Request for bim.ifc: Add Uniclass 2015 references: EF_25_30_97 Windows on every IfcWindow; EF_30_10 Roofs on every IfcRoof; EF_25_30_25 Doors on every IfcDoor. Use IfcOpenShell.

First a look at what the model holds.

```python
import ifcopenshell

model = ifcopenshell.open("bim.ifc")
print(model.schema)
print("classifications:", [c.Name for c in model.by_type("IfcClassification")])
for ifc_class in ("IfcDoor", "IfcRoof", "IfcStair", "IfcWall", "IfcWindow"):
    print(ifc_class, len(model.by_type(ifc_class)))
```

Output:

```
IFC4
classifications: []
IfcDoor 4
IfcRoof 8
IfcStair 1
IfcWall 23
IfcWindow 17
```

```python
import ifcopenshell
import ifcopenshell.api.classification

model = ifcopenshell.open("bim.ifc")

system = ifcopenshell.api.classification.add_classification(model, classification="Uniclass 2015")

codes = {
    "IfcWindow": ("EF_25_30_97", "Windows"),
    "IfcRoof": ("EF_30_10", "Roofs"),
    "IfcDoor": ("EF_25_30_25", "Doors"),
}
for ifc_class, (code, name) in codes.items():
    products = model.by_type(ifc_class)
    ifcopenshell.api.classification.add_reference(
        model, products=products, classification=system, identification=code, name=name
    )
    print(code, len(products))

model.write("bim_edited.ifc")
```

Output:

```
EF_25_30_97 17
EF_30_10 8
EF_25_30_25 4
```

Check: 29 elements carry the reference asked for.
